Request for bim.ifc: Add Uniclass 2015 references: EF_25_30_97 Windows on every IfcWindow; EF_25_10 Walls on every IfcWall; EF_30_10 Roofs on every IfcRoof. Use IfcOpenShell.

First a look at what the model holds.

```python
import ifcopenshell

model = ifcopenshell.open("bim.ifc")
print(model.schema)
print("classifications:", [c.Name for c in model.by_type("IfcClassification")])
for ifc_class in ("IfcDoor", "IfcRoof", "IfcStair", "IfcWall", "IfcWindow"):
    print(ifc_class, len(model.by_type(ifc_class)))
```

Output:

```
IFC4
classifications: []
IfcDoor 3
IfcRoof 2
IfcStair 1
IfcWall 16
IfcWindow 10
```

```python
import ifcopenshell
import ifcopenshell.api.classification

model = ifcopenshell.open("bim.ifc")

system = ifcopenshell.api.classification.add_classification(model, classification="Uniclass 2015")

codes = {
    "IfcWindow": ("EF_25_30_97", "Windows"),
    "IfcWall": ("EF_25_10", "Walls"),
    "IfcRoof": ("EF_30_10", "Roofs"),
}
for ifc_class, (code, name) in codes.items():
    products = model.by_type(ifc_class)
    ifcopenshell.api.classification.add_reference(
        model, products=products, classification=system, identification=code, name=name
    )
    print(code, len(products))

model.write("bim-out.ifc")
```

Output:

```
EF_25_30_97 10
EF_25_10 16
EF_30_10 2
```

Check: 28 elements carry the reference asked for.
